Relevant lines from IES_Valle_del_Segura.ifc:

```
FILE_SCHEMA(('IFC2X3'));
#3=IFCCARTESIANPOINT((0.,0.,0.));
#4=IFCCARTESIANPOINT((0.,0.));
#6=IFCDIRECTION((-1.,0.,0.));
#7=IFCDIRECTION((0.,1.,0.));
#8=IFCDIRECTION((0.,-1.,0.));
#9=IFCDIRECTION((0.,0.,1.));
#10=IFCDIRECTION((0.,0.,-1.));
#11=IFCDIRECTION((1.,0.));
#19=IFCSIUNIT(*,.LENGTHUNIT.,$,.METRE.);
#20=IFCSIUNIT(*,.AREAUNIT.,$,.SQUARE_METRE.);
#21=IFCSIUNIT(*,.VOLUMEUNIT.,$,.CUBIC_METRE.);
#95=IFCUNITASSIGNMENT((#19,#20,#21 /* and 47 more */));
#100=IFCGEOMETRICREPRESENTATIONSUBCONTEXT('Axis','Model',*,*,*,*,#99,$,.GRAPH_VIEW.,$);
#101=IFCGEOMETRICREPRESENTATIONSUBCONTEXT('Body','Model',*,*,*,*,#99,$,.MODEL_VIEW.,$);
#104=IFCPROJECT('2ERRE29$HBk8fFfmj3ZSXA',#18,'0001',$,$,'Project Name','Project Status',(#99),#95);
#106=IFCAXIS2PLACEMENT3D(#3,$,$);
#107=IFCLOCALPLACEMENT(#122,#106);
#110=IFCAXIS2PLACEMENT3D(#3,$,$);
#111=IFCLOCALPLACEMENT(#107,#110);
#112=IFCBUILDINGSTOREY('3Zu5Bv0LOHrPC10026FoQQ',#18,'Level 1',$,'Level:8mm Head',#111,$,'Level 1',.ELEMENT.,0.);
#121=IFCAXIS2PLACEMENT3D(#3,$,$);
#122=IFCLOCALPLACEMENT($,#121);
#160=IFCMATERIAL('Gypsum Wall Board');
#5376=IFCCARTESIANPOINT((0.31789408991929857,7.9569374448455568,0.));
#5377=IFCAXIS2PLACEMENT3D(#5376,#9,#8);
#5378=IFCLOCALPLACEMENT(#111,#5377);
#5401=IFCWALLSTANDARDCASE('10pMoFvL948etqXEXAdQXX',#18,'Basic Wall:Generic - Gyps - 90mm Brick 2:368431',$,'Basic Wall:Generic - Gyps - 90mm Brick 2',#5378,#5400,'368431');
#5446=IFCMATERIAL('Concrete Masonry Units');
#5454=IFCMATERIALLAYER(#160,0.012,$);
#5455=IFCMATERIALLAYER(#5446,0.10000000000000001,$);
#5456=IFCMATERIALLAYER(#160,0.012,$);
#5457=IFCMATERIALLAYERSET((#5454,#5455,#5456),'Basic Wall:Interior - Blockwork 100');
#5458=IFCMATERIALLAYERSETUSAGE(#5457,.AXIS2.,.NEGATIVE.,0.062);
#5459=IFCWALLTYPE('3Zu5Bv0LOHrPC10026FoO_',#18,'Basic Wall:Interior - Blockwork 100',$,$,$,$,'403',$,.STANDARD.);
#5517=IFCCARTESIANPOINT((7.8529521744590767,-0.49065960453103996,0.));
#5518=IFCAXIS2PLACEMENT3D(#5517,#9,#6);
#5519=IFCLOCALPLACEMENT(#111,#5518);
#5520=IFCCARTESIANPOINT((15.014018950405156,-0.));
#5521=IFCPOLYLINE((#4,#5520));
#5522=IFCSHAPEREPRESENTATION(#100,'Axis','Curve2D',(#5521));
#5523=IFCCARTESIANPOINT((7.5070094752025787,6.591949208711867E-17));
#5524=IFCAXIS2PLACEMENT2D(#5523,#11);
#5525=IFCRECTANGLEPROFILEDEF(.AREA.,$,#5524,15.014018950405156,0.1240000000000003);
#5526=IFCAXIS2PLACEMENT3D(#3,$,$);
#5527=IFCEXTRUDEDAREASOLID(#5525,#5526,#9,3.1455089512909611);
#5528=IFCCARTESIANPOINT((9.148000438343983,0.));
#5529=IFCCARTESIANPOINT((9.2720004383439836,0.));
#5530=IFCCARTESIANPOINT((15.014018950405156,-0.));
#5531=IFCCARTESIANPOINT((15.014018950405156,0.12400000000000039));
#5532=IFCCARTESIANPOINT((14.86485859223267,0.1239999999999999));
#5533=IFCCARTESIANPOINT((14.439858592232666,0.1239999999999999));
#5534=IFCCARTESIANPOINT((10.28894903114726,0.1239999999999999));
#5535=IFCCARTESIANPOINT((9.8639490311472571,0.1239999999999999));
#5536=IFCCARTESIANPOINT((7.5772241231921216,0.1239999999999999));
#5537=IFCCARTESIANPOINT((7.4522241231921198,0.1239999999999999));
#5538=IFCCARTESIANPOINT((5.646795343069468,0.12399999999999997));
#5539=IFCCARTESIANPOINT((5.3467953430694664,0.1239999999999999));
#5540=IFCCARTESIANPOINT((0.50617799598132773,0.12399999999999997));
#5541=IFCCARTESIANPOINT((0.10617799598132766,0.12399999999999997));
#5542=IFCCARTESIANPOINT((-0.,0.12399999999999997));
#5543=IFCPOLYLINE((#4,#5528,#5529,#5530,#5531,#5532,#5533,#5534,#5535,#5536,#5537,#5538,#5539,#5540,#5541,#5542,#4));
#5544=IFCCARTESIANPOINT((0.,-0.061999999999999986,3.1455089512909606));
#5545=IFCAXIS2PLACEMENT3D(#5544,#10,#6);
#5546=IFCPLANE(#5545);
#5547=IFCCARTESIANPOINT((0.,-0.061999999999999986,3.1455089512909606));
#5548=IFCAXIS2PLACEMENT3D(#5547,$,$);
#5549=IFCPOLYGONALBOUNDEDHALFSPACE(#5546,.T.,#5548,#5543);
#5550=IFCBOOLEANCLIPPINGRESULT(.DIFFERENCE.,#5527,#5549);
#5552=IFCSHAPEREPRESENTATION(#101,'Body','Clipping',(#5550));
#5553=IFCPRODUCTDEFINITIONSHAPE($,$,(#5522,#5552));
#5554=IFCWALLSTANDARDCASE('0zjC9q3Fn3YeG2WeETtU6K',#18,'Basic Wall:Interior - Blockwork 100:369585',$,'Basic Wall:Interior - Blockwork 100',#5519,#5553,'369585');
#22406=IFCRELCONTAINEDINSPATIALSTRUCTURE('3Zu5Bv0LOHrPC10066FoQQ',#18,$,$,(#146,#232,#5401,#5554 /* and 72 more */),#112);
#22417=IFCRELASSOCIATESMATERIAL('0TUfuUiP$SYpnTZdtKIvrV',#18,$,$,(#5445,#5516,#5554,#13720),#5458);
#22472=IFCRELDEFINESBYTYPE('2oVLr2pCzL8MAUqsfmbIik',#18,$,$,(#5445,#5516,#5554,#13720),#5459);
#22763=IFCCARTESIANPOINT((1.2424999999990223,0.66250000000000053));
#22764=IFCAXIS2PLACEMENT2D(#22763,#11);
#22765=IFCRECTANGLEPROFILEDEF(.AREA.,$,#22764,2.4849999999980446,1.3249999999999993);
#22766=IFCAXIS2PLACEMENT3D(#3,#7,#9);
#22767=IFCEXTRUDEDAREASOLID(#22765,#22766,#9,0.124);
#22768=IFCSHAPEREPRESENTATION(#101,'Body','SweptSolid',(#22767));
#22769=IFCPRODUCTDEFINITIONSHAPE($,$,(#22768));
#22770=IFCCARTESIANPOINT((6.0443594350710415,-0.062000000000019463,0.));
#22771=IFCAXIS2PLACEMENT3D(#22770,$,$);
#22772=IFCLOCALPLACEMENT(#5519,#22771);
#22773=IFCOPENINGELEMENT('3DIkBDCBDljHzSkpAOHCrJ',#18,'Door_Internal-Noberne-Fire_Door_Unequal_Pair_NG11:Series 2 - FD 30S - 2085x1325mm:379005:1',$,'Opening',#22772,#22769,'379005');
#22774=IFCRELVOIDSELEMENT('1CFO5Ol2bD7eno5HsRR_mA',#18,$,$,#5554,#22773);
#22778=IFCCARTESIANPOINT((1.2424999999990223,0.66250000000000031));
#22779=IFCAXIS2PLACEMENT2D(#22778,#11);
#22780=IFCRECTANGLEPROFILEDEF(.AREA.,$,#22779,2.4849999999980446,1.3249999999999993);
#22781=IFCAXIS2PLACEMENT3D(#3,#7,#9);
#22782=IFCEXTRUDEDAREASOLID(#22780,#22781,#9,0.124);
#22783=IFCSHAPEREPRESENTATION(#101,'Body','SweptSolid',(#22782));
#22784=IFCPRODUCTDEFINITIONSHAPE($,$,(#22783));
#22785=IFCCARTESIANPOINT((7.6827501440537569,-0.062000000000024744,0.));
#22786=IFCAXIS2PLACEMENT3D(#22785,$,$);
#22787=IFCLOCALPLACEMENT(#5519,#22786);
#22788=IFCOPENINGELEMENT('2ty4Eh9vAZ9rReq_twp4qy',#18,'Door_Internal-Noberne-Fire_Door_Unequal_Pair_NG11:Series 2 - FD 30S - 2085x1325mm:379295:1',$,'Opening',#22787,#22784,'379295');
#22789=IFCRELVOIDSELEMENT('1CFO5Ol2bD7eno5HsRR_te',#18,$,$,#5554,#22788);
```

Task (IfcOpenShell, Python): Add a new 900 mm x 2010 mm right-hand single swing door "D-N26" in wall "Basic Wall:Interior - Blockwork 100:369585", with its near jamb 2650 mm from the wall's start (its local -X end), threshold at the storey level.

```python
import numpy as np
import ifcopenshell
import ifcopenshell.api.feature
import ifcopenshell.api.geometry
import ifcopenshell.api.root
import ifcopenshell.api.spatial
import ifcopenshell.api.type
import ifcopenshell.geom
import ifcopenshell.util.element
import ifcopenshell.util.placement
import ifcopenshell.util.representation
import ifcopenshell.util.shape
import ifcopenshell.util.unit

model = ifcopenshell.open("IES_Valle_del_Segura.ifc")
unit_scale = ifcopenshell.util.unit.calculate_unit_scale(model)
settings = ifcopenshell.geom.settings()


def volume(element):
    """Net volume in cubic metres, openings subtracted."""
    shape = ifcopenshell.geom.create_shape(settings, element)
    return ifcopenshell.util.shape.get_volume(shape.geometry)


wall = model.by_guid("0zjC9q3Fn3YeG2WeETtU6K")
storey = ifcopenshell.util.element.get_container(wall, ifc_class="IfcBuildingStorey")
context = ifcopenshell.util.representation.get_context(model, "Model", "Body", "MODEL_VIEW")
before = volume(wall)

width, height, from_end, sill = 0.9, 2.01, 2.65, 0.0  # metres

# The wall runs along its own X axis, and the end named is its -X end.
wall_shape = ifcopenshell.geom.create_shape(settings, wall)
x, y, z = ifcopenshell.util.shape.get_vertices(wall_shape.geometry).T
start = x.min() + from_end
face, thickness = float(y.min()), float(y.max() - y.min())
wall_matrix = ifcopenshell.util.placement.get_local_placement(wall.ObjectPlacement)
level = ifcopenshell.util.placement.get_local_placement(storey.ObjectPlacement)[2, 3]


def in_wall(x, y):
    """Placement at x, y metres in the wall's axes, at sill height."""
    matrix = wall_matrix.copy()
    matrix[:, 3] = wall_matrix @ np.array([x / unit_scale, y / unit_scale, 0.0, 1.0])
    matrix[2, 3] = level + sill / unit_scale
    return matrix


# Opening: a box that overshoots both wall faces by 50 mm.
opening = ifcopenshell.api.root.create_entity(model, ifc_class="IfcOpeningElement")
box = ifcopenshell.api.geometry.add_wall_representation(
    model, context=context, length=width, height=height, thickness=thickness + 0.1
)
ifcopenshell.api.geometry.assign_representation(model, product=opening, representation=box)
ifcopenshell.api.geometry.edit_object_placement(model, product=opening, matrix=in_wall(start, face - 0.05), is_si=False)
ifcopenshell.api.feature.add_feature(model, feature=opening, element=wall)

door = ifcopenshell.api.root.create_entity(model, ifc_class="IfcDoor", name="D-N26")
door.OverallWidth, door.OverallHeight = width / unit_scale, height / unit_scale
body = ifcopenshell.api.geometry.add_door_representation(
    model,
    context=context,
    overall_width=door.OverallWidth,
    overall_height=door.OverallHeight,
    operation_type="SINGLE_SWING_RIGHT",
    lining_properties={"LiningDepth": thickness / unit_scale, "ThresholdDepth": thickness / unit_scale},
)
ifcopenshell.api.geometry.assign_representation(model, product=door, representation=body)
ifcopenshell.api.spatial.assign_container(model, products=[door], relating_structure=storey)
fills = ifcopenshell.api.feature.add_filling(model, opening=opening, element=door)
fills.OwnerHistory = door.OwnerHistory  # required in IFC2X3

# IFC2X3 keeps the operation on the door style.
style = ifcopenshell.api.root.create_entity(model, ifc_class="IfcDoorStyle", name="D-N26")
style.OperationType, style.ConstructionType = "SINGLE_SWING_RIGHT", "NOTDEFINED"
style.ParameterTakesPrecedence = style.Sizeable = False
ifcopenshell.api.type.assign_type(model, related_objects=[door], relating_type=style)

# The lining spans the wall, so the door starts at the wall face.
ifcopenshell.api.geometry.edit_object_placement(model, product=door, matrix=in_wall(start, face), is_si=False)

after = volume(wall)

print(f"wall volume {before:.3f} -> {after:.3f} m3")

model.write("IES_Valle_del_Segura_v2.ifc")
```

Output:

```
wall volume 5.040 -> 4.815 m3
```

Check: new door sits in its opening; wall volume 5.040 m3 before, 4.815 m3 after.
